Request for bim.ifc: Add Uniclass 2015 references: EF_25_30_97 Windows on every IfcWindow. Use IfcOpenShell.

First a look at what the model holds.

```python
import ifcopenshell

model = ifcopenshell.open("bim.ifc")
print(model.schema)
print("classifications:", [c.Name for c in model.by_type("IfcClassification")])
for ifc_class in ("IfcDoor", "IfcRoof", "IfcStair", "IfcWall", "IfcWindow"):
    print(ifc_class, len(model.by_type(ifc_class)))
```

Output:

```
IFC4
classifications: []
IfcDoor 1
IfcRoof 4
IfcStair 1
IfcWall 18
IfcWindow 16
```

```python
import ifcopenshell
import ifcopenshell.api.classification

model = ifcopenshell.open("bim.ifc")

system = ifcopenshell.api.classification.add_classification(model, classification="Uniclass 2015")

codes = {
    "IfcWindow": ("EF_25_30_97", "Windows"),
}
for ifc_class, (code, name) in codes.items():
    products = model.by_type(ifc_class)
    ifcopenshell.api.classification.add_reference(
        model, products=products, classification=system, identification=code, name=name
    )
    print(code, len(products))

model.write("bim_v2.ifc")
```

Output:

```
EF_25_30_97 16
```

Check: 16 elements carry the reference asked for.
